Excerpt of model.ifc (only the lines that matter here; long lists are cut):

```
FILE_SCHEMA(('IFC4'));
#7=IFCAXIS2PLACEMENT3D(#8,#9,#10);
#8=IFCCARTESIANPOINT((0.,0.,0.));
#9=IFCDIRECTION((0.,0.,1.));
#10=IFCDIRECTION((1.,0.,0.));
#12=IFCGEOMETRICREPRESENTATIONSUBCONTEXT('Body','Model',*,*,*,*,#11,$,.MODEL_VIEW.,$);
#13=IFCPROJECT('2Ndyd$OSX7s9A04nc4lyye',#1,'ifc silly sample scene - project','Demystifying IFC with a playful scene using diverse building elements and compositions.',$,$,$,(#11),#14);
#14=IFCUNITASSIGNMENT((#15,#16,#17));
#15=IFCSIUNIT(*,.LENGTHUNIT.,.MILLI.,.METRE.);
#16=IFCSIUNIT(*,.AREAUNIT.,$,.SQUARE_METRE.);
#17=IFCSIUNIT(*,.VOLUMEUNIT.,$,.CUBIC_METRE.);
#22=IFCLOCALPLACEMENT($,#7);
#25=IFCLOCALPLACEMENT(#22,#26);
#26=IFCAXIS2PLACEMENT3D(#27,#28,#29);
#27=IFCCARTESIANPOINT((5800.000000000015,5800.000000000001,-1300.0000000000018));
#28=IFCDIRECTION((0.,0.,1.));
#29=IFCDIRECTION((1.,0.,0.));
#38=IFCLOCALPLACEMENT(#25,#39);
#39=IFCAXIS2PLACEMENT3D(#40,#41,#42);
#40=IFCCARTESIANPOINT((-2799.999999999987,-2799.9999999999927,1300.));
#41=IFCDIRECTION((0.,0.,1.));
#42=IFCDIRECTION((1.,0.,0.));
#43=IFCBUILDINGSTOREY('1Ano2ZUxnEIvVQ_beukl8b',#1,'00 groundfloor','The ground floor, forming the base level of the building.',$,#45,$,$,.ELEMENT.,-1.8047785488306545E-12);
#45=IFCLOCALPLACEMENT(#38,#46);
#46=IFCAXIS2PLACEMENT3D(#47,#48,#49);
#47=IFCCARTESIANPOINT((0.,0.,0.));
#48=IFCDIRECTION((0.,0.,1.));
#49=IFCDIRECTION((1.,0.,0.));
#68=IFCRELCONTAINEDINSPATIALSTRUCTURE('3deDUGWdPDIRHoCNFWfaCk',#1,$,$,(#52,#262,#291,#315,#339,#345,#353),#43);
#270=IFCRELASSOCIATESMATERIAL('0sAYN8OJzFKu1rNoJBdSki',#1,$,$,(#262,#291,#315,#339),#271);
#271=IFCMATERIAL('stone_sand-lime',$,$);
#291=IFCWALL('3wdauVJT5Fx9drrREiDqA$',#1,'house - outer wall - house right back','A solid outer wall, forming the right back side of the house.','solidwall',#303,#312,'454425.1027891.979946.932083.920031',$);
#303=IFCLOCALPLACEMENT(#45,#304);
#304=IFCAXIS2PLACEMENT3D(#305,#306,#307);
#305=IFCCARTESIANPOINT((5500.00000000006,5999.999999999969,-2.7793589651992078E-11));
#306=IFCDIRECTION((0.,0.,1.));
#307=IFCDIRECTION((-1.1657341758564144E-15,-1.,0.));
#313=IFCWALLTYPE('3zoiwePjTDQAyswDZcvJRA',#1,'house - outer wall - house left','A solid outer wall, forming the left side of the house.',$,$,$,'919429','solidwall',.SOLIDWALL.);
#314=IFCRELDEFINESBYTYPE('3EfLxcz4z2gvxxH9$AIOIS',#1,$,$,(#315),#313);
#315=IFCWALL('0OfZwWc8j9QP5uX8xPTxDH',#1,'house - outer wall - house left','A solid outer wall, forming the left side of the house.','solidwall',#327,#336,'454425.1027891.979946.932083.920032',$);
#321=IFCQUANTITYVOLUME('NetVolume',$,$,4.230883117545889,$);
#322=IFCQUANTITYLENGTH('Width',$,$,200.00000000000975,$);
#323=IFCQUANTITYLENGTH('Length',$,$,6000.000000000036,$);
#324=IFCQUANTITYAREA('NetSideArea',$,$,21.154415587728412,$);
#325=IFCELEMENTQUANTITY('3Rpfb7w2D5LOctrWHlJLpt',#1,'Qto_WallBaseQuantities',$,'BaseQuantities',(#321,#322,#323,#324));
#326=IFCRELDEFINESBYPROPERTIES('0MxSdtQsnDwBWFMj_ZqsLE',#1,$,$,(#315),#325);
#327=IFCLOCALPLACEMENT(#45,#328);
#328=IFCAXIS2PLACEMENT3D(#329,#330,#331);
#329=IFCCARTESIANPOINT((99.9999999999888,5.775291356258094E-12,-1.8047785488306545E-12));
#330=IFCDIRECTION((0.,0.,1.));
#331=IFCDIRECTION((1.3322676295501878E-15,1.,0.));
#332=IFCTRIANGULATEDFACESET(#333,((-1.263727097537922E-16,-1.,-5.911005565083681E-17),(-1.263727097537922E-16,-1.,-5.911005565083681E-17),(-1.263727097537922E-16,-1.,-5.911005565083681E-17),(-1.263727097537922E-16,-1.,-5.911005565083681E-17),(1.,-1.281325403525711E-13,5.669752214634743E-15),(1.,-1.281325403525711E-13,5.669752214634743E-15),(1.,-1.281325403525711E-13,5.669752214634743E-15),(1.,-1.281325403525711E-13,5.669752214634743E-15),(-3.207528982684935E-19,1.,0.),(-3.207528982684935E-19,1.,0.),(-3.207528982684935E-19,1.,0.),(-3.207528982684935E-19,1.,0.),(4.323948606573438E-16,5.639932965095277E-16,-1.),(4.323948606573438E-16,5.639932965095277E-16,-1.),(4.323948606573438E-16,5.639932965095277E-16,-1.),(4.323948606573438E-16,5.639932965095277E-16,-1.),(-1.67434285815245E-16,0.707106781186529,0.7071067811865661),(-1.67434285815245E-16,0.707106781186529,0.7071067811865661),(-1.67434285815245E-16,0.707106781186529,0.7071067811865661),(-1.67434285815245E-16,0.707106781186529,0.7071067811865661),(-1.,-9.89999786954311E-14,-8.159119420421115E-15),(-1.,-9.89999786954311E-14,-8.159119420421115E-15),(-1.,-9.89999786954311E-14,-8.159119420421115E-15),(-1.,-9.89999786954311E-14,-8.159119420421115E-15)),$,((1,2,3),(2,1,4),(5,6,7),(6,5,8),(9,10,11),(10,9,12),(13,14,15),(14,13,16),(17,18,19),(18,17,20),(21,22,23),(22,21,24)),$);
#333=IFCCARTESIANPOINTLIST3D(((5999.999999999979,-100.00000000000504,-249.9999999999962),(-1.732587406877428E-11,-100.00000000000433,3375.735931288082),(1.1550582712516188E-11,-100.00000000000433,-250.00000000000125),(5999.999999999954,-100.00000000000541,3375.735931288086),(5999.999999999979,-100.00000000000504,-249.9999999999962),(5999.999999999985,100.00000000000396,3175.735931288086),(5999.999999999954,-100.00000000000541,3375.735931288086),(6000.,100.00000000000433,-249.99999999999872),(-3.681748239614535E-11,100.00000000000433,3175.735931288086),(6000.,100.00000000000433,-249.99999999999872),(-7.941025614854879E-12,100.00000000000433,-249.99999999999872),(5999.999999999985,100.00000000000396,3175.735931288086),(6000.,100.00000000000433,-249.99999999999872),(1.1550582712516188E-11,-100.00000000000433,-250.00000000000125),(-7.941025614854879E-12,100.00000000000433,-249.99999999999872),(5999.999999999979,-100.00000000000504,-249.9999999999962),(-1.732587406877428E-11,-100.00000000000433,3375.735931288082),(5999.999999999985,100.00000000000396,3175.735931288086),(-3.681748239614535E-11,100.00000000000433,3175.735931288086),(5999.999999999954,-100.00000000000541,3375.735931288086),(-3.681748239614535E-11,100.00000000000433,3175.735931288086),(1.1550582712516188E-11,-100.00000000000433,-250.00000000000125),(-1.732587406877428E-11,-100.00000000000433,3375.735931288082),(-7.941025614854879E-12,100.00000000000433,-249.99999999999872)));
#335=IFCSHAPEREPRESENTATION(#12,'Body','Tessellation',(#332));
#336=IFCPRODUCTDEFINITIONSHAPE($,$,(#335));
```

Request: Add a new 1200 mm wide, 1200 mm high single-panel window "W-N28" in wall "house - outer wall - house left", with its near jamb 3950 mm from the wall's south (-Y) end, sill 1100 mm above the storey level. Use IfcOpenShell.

```python
import numpy as np
import ifcopenshell
import ifcopenshell.api.feature
import ifcopenshell.api.geometry
import ifcopenshell.api.pset
import ifcopenshell.api.root
import ifcopenshell.api.spatial
import ifcopenshell.geom
import ifcopenshell.util.element
import ifcopenshell.util.placement
import ifcopenshell.util.representation
import ifcopenshell.util.shape
import ifcopenshell.util.unit

model = ifcopenshell.open("model.ifc")
unit_scale = ifcopenshell.util.unit.calculate_unit_scale(model)
area_scale = ifcopenshell.util.unit.calculate_unit_scale(model, "AREAUNIT")
volume_scale = ifcopenshell.util.unit.calculate_unit_scale(model, "VOLUMEUNIT")
settings = ifcopenshell.geom.settings()


def volume(element):
    """Net volume in cubic metres, openings subtracted."""
    shape = ifcopenshell.geom.create_shape(settings, element)
    return ifcopenshell.util.shape.get_volume(shape.geometry)


wall = model.by_id(315)
storey = ifcopenshell.util.element.get_container(wall, ifc_class="IfcBuildingStorey")
context = ifcopenshell.util.representation.get_context(model, "Model", "Body", "MODEL_VIEW")
before = volume(wall)

width, height, from_end, sill = 1.2, 1.2, 3.95, 1.1  # metres

# The wall runs along its own X axis, and the end named is its -X end.
wall_shape = ifcopenshell.geom.create_shape(settings, wall)
x, y, z = ifcopenshell.util.shape.get_vertices(wall_shape.geometry).T
start = x.min() + from_end
face, thickness = float(y.min()), float(y.max() - y.min())
wall_matrix = ifcopenshell.util.placement.get_local_placement(wall.ObjectPlacement)
level = ifcopenshell.util.placement.get_local_placement(storey.ObjectPlacement)[2, 3]


def in_wall(x, y):
    """Placement at x, y metres in the wall's axes, at sill height."""
    matrix = wall_matrix.copy()
    matrix[:, 3] = wall_matrix @ np.array([x / unit_scale, y / unit_scale, 0.0, 1.0])
    matrix[2, 3] = level + sill / unit_scale
    return matrix


# Opening: a box that overshoots both wall faces by 50 mm.
opening = ifcopenshell.api.root.create_entity(model, ifc_class="IfcOpeningElement", predefined_type="OPENING")
box = ifcopenshell.api.geometry.add_wall_representation(
    model, context=context, length=width, height=height, thickness=thickness + 0.1
)
ifcopenshell.api.geometry.assign_representation(model, product=opening, representation=box)
ifcopenshell.api.geometry.edit_object_placement(model, product=opening, matrix=in_wall(start, face - 0.05), is_si=False)
ifcopenshell.api.feature.add_feature(model, feature=opening, element=wall)

window = ifcopenshell.api.root.create_entity(model, ifc_class="IfcWindow", name="W-N28", predefined_type="WINDOW")
window.OverallWidth, window.OverallHeight = width / unit_scale, height / unit_scale
window.PartitioningType = "SINGLE_PANEL"
body = ifcopenshell.api.geometry.add_window_representation(
    model,
    context=context,
    overall_width=window.OverallWidth,
    overall_height=window.OverallHeight,
    partition_type="SINGLE_PANEL",
)
ifcopenshell.api.geometry.assign_representation(model, product=window, representation=body)
ifcopenshell.api.spatial.assign_container(model, products=[window], relating_structure=storey)
ifcopenshell.api.feature.add_filling(model, opening=opening, element=window)

# Centre the window in the wall's thickness.
ifcopenshell.api.geometry.edit_object_placement(model, product=window, matrix=in_wall(start, face), is_si=False)
window_shape = ifcopenshell.geom.create_shape(settings, window)
depth = ifcopenshell.util.shape.get_vertices(window_shape.geometry)[:, 1]
offset = face + thickness / 2 - (depth.min() + depth.max()) / 2
ifcopenshell.api.geometry.edit_object_placement(model, product=window, matrix=in_wall(start, offset), is_si=False)

after = volume(wall)

# Update the wall's stored quantities.
qto = model.by_id(ifcopenshell.util.element.get_pset(wall, "Qto_WallBaseQuantities", should_inherit=False)["id"])
ifcopenshell.api.pset.edit_qto(model, qto=qto, properties={
    "NetVolume": after / volume_scale,
    "NetSideArea": after / thickness / area_scale,
})

print(f"wall volume {before:.3f} -> {after:.3f} m3")

model.write("model_edited.ifc")
```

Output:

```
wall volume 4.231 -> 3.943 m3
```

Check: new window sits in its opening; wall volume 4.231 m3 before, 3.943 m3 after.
